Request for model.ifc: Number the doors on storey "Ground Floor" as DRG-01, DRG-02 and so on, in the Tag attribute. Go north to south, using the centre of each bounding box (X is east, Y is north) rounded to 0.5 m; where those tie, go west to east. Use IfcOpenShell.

First a look at what the model holds.

```python
import ifcopenshell
import ifcopenshell.util.element
import ifcopenshell.util.placement

model = ifcopenshell.open("model.ifc")
print(model.schema)
storey = next(s for s in model.by_type("IfcBuildingStorey") if s.Name == "Ground Floor")
doors = [e for e in ifcopenshell.util.element.get_decomposition(storey) if e.is_a("IfcDoor")]
for e in sorted(doors, key=lambda e: e.id()):
    origin = ifcopenshell.util.placement.get_local_placement(e.ObjectPlacement)[:3, 3]
    print(e.id(), e.Tag, e.Name, origin.round(2) + 0.0, sep=" | ")
```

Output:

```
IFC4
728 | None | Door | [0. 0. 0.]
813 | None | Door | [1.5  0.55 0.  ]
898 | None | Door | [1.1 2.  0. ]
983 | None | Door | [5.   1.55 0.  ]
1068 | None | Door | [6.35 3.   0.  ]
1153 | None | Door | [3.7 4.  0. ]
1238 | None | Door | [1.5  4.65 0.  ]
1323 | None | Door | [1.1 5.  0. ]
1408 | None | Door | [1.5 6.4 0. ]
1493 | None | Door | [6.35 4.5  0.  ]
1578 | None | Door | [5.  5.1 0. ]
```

```python
import ifcopenshell
import ifcopenshell.geom
import ifcopenshell.util.element
import ifcopenshell.util.shape

model = ifcopenshell.open("model.ifc")
settings = ifcopenshell.geom.settings()
settings.set("use-world-coords", True)


def centre(element):
    shape = ifcopenshell.geom.create_shape(settings, element)
    return ifcopenshell.util.shape.get_bbox_centroid(shape.geometry)


storey = next(s for s in model.by_type("IfcBuildingStorey") if s.Name == "Ground Floor")
doors = [e for e in ifcopenshell.util.element.get_decomposition(storey) if e.is_a("IfcDoor")]

# Insertion points can sit at a corner or the storey origin, so sort by the geometry (in metres).
centres = {e: centre(e) for e in doors}
doors.sort(key=lambda e: (-round(centres[e][1] / 0.5), centres[e][0]))

for i, e in enumerate(doors, start=1):
    number = f"DRG-{i:02d}"
    e.Tag = number
    print(e.id(), number)

model.write("model_updated.ifc")
```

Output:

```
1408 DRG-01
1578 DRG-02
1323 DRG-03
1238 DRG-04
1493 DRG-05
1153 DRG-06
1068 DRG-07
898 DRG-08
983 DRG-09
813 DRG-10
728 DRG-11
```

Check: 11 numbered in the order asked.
